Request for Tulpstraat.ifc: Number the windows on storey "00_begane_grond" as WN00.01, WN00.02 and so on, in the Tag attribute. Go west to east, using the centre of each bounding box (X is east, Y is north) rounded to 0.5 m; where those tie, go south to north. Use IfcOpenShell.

First a look at what the model holds.

```python
import ifcopenshell
import ifcopenshell.util.element
import ifcopenshell.util.placement

model = ifcopenshell.open("Tulpstraat.ifc")
print(model.schema)
storey = next(s for s in model.by_type("IfcBuildingStorey") if s.Name == "00_begane_grond")
windows = [e for e in ifcopenshell.util.element.get_decomposition(storey) if e.is_a("IfcWindow")]
for e in sorted(windows, key=lambda e: e.id()):
    origin = ifcopenshell.util.placement.get_local_placement(e.ObjectPlacement)[:3, 3]
    print(e.id(), e.Tag, e.Name, origin.round(2) + 0.0, sep=" | ")
```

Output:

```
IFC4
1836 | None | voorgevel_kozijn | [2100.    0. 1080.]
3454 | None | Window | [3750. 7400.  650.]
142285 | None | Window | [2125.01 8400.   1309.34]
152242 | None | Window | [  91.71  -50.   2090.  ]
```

```python
import ifcopenshell
import ifcopenshell.geom
import ifcopenshell.util.element
import ifcopenshell.util.shape

model = ifcopenshell.open("Tulpstraat.ifc")
settings = ifcopenshell.geom.settings()
settings.set("use-world-coords", True)


def centre(element):
    shape = ifcopenshell.geom.create_shape(settings, element)
    return ifcopenshell.util.shape.get_bbox_centroid(shape.geometry)


storey = next(s for s in model.by_type("IfcBuildingStorey") if s.Name == "00_begane_grond")
windows = [e for e in ifcopenshell.util.element.get_decomposition(storey) if e.is_a("IfcWindow")]

# Insertion points can sit at a corner or the storey origin, so sort by the geometry (in metres).
centres = {e: centre(e) for e in windows}
windows.sort(key=lambda e: (round(centres[e][0] / 0.5), centres[e][1]))

for i, e in enumerate(windows, start=1):
    number = f"WN00.{i:02d}"
    e.Tag = number
    print(e.id(), number)

model.write("Tulpstraat_rev.ifc")
```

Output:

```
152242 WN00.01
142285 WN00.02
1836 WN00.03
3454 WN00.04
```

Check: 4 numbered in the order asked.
